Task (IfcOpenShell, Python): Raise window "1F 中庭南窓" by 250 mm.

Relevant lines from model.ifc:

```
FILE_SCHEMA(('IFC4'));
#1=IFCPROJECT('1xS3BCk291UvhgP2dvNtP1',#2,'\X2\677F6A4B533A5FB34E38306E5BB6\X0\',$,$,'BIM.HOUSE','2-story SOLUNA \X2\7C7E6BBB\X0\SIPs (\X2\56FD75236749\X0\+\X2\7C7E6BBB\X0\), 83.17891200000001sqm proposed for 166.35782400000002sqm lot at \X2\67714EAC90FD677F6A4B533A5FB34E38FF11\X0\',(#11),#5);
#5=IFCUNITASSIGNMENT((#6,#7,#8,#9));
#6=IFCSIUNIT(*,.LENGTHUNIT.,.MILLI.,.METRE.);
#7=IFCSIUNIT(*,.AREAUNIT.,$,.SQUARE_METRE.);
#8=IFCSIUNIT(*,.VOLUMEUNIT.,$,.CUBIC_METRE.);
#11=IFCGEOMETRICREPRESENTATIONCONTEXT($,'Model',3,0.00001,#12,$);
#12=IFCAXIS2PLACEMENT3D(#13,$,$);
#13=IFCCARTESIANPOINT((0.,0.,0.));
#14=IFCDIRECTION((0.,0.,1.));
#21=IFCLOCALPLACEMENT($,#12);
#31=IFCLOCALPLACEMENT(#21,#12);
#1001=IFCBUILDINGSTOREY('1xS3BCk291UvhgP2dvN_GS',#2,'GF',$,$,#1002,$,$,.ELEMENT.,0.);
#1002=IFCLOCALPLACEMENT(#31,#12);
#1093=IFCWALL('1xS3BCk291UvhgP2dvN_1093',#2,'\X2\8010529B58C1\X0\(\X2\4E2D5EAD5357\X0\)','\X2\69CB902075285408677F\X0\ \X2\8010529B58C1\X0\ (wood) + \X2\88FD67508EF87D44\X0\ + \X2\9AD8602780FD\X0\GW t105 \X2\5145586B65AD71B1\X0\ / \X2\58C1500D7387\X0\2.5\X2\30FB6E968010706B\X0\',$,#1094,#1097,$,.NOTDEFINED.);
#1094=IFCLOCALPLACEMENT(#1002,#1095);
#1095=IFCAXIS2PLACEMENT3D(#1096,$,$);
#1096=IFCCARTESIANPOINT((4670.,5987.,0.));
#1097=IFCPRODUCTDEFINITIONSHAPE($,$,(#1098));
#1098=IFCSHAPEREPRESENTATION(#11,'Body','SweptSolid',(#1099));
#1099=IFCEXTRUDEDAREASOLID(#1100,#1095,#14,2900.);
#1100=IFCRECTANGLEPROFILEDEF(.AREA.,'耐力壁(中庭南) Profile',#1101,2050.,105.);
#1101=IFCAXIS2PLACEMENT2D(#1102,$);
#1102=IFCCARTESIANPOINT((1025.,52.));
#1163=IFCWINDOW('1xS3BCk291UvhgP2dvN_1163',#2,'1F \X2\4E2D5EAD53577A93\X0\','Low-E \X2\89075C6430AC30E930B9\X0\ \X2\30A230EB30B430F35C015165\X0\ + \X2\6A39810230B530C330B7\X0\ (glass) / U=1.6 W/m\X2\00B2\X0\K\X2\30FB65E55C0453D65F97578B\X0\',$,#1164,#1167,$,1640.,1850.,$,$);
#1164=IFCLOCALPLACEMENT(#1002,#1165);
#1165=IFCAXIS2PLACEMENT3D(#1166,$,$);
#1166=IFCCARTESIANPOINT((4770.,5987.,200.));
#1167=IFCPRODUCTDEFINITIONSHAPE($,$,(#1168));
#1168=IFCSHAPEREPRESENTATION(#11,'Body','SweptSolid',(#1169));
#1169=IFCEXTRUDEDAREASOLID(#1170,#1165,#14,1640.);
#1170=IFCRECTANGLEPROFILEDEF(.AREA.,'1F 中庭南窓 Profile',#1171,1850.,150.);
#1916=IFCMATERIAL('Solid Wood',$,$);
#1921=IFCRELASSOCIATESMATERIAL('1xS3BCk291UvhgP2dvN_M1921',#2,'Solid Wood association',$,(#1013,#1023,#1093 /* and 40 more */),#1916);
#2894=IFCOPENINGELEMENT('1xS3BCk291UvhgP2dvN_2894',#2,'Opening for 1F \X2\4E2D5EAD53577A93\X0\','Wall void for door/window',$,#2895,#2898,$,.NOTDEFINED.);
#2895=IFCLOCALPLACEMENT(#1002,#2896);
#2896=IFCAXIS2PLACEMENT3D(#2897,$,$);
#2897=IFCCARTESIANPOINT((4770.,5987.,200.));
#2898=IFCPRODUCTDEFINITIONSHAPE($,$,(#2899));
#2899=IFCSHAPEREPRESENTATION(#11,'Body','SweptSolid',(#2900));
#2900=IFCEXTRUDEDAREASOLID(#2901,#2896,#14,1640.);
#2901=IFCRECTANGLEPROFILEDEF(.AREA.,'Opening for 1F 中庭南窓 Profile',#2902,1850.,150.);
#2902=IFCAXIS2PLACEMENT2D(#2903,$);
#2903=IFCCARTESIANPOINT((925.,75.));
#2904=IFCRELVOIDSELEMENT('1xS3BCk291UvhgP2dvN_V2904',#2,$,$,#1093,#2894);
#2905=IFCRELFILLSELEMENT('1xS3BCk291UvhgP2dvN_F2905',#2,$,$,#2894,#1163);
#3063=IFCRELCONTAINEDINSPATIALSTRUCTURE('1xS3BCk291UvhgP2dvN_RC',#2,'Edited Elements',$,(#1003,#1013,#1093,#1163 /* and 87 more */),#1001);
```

```python
import numpy as np
import ifcopenshell
import ifcopenshell.api.geometry
import ifcopenshell.util.placement
import ifcopenshell.util.unit

model = ifcopenshell.open("model.ifc")
unit_scale = ifcopenshell.util.unit.calculate_unit_scale(model)

window = model.by_id(1163)
opening = window.FillsVoids[0].RelatingOpeningElement
dz = 0.25 / unit_scale

shift = np.array([0.0, 0.0, dz])
# The window is not placed relative to its opening, so move both.
for product in (opening, window):
    matrix = ifcopenshell.util.placement.get_local_placement(product.ObjectPlacement)
    matrix[:3, 3] += shift
    ifcopenshell.api.geometry.edit_object_placement(model, product=product, matrix=matrix, is_si=False)

print(f"moved by {dz * unit_scale:+.3f} m")

model.write("model_updated.ifc")
```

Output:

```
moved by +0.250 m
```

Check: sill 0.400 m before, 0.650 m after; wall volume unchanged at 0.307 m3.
